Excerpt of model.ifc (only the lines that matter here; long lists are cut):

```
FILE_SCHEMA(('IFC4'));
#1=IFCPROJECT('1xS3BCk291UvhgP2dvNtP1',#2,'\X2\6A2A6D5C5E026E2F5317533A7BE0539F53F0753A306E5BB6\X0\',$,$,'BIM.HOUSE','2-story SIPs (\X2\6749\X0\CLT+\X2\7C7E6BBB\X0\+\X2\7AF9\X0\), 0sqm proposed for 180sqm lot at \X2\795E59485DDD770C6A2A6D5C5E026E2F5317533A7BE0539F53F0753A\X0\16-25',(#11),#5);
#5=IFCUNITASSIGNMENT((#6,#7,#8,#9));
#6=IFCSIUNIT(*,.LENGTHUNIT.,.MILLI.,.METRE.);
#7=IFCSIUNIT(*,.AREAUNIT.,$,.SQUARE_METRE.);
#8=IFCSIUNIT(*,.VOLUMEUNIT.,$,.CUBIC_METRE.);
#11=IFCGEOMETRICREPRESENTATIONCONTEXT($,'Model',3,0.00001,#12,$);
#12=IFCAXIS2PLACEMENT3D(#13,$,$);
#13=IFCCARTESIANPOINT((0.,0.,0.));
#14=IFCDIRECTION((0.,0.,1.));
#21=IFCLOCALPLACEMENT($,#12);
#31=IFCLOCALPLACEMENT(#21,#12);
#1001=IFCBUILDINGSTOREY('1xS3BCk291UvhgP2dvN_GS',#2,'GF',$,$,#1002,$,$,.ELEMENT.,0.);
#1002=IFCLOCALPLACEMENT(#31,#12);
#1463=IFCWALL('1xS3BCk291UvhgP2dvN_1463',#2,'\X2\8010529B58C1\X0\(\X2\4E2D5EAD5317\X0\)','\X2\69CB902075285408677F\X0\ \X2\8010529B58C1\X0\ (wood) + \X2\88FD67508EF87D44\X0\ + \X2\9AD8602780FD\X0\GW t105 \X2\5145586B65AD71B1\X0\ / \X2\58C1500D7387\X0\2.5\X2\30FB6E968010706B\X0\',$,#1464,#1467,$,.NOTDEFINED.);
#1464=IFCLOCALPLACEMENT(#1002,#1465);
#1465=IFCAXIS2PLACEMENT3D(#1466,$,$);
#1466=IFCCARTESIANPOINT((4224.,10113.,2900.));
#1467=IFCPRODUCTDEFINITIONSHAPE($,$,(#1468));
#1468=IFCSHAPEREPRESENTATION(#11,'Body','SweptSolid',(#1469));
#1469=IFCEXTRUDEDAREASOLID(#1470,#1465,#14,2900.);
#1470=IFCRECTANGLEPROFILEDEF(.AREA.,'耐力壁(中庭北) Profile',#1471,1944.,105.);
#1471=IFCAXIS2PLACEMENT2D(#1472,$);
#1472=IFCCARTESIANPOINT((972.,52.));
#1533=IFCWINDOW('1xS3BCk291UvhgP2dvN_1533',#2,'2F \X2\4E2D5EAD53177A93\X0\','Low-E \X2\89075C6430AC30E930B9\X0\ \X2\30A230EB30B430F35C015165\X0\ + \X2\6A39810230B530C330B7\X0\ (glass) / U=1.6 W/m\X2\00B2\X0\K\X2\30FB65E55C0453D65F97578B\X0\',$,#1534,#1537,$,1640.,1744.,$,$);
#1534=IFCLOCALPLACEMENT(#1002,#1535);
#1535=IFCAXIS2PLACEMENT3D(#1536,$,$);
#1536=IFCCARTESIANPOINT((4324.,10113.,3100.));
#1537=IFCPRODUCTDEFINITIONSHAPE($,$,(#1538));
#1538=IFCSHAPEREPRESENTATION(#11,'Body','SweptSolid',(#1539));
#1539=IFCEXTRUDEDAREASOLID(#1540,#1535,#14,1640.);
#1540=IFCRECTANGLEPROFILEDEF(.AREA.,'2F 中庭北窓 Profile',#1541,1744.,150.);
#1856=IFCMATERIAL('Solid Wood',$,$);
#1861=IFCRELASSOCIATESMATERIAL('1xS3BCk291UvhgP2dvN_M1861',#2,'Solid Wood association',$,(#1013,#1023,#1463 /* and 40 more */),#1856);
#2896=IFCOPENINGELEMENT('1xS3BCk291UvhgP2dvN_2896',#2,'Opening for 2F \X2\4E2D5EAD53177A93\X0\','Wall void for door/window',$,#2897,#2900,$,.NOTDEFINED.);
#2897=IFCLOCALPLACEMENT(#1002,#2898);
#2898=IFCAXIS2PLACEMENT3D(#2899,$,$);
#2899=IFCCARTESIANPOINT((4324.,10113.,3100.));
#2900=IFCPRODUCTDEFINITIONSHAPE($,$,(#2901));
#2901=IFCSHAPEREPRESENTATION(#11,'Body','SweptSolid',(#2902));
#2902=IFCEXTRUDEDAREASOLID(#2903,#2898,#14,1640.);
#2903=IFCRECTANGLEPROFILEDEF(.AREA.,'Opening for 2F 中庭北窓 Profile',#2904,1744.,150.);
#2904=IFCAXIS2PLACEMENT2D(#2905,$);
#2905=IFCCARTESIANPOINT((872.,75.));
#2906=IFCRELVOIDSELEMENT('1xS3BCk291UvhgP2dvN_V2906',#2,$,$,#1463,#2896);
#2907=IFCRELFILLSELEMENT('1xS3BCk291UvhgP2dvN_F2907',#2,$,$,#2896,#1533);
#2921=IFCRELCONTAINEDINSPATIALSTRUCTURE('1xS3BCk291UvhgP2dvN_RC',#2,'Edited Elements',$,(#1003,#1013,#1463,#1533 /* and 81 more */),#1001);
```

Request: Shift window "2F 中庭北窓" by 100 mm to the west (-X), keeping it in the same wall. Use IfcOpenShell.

```python
import ifcopenshell
import ifcopenshell.api.geometry
import ifcopenshell.util.placement
import ifcopenshell.util.unit

model = ifcopenshell.open("model.ifc")
unit_scale = ifcopenshell.util.unit.calculate_unit_scale(model)

window = model.by_guid("1xS3BCk291UvhgP2dvN_1533")
opening = window.FillsVoids[0].RelatingOpeningElement
wall = opening.VoidsElements[0].RelatingBuildingElement

wall_matrix = ifcopenshell.util.placement.get_local_placement(wall.ObjectPlacement)
shift = wall_matrix[:3, 0] * -0.1 / unit_scale
before = ifcopenshell.util.placement.get_local_placement(window.ObjectPlacement)[:3, 3].copy()

# The window is not placed relative to its opening, so move both.
for product in (opening, window):
    matrix = ifcopenshell.util.placement.get_local_placement(product.ObjectPlacement)
    matrix[:3, 3] += shift
    ifcopenshell.api.geometry.edit_object_placement(model, product=product, matrix=matrix, is_si=False)

after = ifcopenshell.util.placement.get_local_placement(window.ObjectPlacement)[:3, 3]
print("window moved by", (after - before).round(3) + 0.0)

model.write("model_edited.ifc")
```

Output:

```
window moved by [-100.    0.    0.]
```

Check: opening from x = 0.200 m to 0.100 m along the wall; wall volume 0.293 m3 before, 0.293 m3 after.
